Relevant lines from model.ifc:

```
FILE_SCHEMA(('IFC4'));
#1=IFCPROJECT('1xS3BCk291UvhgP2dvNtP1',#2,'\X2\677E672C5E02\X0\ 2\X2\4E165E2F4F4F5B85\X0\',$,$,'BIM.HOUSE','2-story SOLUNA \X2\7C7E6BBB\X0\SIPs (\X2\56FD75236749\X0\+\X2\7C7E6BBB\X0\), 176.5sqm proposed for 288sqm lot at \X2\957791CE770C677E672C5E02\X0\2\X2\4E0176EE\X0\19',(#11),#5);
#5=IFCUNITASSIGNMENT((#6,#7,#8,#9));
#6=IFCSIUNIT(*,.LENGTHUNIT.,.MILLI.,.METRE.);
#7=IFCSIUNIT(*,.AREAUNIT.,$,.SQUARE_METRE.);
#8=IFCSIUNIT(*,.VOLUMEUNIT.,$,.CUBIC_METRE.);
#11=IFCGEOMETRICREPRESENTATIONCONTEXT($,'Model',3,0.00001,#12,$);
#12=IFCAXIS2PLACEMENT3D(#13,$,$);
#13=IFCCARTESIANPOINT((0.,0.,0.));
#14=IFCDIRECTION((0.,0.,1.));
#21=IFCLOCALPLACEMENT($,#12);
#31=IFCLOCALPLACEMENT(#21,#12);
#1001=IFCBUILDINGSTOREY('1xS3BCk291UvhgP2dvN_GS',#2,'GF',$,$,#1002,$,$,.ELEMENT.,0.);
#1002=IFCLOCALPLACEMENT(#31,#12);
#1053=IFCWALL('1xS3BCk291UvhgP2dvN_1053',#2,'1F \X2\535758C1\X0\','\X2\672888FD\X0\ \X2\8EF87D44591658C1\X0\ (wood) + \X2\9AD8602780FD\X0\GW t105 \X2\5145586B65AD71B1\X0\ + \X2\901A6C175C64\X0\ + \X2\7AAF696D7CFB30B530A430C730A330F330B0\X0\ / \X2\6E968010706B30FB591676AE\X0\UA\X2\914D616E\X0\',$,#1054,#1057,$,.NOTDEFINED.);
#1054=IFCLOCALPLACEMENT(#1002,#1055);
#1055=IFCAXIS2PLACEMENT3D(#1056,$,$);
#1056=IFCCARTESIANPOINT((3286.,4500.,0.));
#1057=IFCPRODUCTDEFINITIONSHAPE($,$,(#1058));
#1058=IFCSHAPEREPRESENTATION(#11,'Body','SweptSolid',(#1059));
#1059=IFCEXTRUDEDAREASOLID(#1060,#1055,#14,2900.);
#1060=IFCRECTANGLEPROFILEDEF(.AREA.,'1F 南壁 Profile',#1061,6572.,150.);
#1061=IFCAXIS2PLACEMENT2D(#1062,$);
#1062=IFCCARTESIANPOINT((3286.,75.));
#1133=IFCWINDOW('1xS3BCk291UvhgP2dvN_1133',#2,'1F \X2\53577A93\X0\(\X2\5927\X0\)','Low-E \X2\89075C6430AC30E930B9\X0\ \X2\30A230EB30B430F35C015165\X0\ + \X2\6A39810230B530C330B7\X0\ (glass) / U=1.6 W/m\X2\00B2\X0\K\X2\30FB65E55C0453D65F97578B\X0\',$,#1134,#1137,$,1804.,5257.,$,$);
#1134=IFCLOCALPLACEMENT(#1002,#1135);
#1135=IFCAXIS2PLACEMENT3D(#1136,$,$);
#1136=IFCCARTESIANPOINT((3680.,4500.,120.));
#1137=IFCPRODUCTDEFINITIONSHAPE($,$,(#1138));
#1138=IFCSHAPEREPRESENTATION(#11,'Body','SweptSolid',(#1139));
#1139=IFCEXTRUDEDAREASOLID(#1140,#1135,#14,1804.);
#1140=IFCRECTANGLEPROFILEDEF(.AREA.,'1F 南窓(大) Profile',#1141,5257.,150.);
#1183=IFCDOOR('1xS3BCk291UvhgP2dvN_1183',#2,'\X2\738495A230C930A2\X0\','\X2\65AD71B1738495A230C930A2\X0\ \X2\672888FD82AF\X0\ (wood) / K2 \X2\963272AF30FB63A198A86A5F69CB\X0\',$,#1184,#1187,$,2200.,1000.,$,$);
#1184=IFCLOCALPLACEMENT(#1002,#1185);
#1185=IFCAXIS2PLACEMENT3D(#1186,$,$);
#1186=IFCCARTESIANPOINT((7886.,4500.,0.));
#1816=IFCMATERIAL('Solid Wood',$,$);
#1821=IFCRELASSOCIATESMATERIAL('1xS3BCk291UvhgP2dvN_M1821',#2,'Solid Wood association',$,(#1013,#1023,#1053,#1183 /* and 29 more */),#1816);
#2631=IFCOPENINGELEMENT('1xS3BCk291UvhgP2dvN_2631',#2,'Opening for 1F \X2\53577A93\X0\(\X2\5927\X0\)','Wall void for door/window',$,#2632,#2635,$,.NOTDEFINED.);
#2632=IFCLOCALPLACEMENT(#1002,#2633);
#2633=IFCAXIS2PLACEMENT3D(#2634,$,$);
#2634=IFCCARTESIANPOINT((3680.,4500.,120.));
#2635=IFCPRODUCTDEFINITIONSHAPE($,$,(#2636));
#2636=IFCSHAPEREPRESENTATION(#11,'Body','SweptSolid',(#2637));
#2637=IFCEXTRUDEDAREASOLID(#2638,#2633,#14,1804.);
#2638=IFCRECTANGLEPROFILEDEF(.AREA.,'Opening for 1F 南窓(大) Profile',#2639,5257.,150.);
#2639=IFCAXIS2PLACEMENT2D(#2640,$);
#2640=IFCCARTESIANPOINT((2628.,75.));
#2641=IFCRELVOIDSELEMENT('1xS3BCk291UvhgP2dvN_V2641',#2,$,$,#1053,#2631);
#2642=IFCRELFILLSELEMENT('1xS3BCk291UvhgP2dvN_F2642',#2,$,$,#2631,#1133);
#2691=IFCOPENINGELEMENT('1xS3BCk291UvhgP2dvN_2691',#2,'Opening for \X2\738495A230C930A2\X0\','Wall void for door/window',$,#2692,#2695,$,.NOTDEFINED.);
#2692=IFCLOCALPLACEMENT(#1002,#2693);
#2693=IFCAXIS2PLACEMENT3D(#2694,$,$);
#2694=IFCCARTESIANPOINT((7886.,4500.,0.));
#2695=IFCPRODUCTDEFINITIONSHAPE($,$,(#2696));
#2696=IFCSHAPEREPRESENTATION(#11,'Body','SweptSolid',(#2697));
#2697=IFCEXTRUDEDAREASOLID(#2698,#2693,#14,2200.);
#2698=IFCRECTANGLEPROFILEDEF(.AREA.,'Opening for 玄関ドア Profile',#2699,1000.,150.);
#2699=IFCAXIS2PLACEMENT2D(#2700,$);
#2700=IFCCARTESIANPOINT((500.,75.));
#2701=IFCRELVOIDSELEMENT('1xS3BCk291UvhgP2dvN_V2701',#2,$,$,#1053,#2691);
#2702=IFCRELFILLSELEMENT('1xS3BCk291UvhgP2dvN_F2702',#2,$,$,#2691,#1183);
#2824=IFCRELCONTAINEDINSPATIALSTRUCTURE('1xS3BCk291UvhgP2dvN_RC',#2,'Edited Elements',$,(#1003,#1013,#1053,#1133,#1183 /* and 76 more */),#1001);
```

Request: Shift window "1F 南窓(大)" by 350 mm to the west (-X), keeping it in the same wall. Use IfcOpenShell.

```python
import ifcopenshell
import ifcopenshell.api.geometry
import ifcopenshell.util.placement
import ifcopenshell.util.unit

model = ifcopenshell.open("model.ifc")
unit_scale = ifcopenshell.util.unit.calculate_unit_scale(model)

window = model.by_id(1133)
opening = window.FillsVoids[0].RelatingOpeningElement
wall = opening.VoidsElements[0].RelatingBuildingElement

wall_matrix = ifcopenshell.util.placement.get_local_placement(wall.ObjectPlacement)
shift = wall_matrix[:3, 0] * -0.35 / unit_scale
before = ifcopenshell.util.placement.get_local_placement(window.ObjectPlacement)[:3, 3].copy()

# The window is not placed relative to its opening, so move both.
for product in (opening, window):
    matrix = ifcopenshell.util.placement.get_local_placement(product.ObjectPlacement)
    matrix[:3, 3] += shift
    ifcopenshell.api.geometry.edit_object_placement(model, product=product, matrix=matrix, is_si=False)

after = ifcopenshell.util.placement.get_local_placement(window.ObjectPlacement)[:3, 3]
print("window moved by", (after - before).round(3) + 0.0)

model.write("model_v2.ifc")
```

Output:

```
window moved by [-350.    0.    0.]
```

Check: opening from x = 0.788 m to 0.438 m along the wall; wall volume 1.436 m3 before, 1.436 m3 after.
